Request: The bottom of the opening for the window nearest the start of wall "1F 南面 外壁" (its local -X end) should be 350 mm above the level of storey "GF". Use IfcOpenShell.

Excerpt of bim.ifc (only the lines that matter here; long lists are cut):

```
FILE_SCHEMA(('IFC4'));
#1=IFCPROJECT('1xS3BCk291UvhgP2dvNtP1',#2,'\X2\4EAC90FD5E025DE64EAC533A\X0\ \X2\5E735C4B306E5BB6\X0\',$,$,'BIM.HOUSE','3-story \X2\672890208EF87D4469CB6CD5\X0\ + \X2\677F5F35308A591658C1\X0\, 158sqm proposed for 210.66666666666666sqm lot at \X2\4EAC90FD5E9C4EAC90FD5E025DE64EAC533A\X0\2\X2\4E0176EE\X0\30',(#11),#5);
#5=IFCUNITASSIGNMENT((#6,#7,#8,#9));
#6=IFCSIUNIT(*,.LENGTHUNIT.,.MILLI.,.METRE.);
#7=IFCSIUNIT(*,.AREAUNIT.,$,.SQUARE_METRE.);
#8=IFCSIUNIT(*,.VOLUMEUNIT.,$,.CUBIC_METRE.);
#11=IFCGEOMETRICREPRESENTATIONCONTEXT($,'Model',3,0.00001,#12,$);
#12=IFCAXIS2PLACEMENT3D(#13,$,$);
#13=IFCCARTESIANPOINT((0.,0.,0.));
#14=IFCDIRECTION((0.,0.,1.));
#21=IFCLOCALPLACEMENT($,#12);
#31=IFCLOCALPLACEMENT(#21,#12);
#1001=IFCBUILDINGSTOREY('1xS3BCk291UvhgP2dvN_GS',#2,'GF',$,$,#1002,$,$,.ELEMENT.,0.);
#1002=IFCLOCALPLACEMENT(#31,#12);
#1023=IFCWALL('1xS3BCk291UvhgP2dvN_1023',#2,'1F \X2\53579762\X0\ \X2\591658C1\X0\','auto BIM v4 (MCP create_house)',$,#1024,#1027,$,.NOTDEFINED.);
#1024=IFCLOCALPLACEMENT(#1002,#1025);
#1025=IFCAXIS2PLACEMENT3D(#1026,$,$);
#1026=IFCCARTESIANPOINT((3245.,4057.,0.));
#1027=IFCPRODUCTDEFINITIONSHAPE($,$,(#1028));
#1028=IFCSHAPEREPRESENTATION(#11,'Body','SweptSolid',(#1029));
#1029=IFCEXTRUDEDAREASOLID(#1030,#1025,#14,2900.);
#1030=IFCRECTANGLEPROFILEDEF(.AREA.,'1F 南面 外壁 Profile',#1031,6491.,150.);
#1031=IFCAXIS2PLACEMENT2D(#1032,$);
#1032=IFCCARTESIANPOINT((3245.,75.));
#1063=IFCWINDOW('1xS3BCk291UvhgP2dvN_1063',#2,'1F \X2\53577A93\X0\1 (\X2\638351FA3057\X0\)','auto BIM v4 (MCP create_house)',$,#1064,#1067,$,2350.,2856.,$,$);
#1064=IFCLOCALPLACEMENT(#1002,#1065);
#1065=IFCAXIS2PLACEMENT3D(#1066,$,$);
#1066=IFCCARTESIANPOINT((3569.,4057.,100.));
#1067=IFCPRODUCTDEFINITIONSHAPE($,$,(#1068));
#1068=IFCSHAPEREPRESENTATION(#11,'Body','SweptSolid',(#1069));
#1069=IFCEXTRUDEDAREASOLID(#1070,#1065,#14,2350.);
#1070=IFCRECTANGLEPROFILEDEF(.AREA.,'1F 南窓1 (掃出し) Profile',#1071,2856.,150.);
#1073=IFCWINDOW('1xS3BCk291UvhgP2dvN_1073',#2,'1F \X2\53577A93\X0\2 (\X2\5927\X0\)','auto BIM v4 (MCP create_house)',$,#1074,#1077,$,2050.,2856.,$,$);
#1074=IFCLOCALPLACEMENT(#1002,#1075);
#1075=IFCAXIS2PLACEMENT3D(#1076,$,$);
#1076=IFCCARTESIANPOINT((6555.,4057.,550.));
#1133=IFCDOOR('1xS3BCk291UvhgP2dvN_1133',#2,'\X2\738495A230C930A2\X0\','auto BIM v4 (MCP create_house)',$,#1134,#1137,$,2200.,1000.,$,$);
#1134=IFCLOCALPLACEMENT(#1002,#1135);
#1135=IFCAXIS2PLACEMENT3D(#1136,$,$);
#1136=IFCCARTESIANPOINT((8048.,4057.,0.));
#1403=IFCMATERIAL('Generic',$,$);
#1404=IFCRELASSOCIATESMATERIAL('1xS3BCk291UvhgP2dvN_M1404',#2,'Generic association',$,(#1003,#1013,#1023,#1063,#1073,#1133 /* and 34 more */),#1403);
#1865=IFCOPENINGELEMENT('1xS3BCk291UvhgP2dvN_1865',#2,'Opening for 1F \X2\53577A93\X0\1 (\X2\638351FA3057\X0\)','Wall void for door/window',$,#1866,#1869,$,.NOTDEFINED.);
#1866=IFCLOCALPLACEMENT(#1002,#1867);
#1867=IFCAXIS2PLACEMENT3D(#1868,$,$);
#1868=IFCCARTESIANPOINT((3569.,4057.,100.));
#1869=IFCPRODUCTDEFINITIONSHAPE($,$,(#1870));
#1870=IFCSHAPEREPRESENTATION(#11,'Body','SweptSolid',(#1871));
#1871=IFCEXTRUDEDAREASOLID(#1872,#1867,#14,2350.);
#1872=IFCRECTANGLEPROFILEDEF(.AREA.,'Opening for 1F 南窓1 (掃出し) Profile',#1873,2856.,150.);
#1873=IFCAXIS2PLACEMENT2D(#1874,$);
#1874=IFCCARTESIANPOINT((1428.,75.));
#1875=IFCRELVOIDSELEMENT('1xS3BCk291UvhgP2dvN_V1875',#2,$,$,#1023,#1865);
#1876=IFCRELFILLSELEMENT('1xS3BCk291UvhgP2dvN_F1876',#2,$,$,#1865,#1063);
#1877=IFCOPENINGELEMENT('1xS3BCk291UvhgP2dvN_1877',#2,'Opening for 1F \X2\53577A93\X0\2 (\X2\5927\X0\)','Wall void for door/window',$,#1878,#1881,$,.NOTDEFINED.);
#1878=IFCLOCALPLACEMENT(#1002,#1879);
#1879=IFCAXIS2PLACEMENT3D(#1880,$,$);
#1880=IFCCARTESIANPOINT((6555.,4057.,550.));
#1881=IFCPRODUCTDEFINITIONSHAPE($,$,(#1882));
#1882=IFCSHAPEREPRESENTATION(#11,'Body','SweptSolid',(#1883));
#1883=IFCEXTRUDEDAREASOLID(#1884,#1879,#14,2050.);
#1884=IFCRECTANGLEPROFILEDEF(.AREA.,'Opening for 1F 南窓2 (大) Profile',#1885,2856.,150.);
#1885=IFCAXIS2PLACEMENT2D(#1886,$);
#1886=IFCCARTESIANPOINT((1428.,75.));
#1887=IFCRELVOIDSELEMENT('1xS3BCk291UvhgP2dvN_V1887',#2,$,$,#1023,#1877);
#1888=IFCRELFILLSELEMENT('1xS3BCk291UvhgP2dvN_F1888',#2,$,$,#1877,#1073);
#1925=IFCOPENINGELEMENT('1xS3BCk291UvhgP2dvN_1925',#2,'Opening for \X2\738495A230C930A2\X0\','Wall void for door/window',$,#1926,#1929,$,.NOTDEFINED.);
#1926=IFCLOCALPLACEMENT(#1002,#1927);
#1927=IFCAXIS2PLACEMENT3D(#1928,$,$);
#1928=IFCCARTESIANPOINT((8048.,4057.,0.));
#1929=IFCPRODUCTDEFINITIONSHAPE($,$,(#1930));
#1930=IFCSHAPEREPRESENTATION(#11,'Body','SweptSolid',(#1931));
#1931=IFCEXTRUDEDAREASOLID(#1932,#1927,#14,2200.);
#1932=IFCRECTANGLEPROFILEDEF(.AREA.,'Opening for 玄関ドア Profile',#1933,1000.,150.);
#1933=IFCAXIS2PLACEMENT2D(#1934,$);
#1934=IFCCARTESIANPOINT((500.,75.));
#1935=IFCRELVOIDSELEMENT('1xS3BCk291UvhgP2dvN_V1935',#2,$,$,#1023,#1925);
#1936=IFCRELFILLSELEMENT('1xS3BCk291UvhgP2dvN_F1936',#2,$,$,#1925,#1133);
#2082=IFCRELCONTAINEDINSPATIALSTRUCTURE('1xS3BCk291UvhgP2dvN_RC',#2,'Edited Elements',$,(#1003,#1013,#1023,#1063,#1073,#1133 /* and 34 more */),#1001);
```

```python
import numpy as np
import ifcopenshell
import ifcopenshell.api.geometry
import ifcopenshell.geom
import ifcopenshell.util.element
import ifcopenshell.util.placement
import ifcopenshell.util.shape
import ifcopenshell.util.unit

model = ifcopenshell.open("bim.ifc")
unit_scale = ifcopenshell.util.unit.calculate_unit_scale(model)

window = model.by_guid("1xS3BCk291UvhgP2dvN_1063")
opening = window.FillsVoids[0].RelatingOpeningElement
storey = ifcopenshell.util.element.get_container(window, ifc_class="IfcBuildingStorey")
level = ifcopenshell.util.placement.get_local_placement(storey.ObjectPlacement)[2, 3]

# The opening's origin need not be at the sill, so measure its lowest point.
shape = ifcopenshell.geom.create_shape(ifcopenshell.geom.settings(), opening)
bottom = ifcopenshell.util.shape.get_shape_bottom_elevation(shape, shape.geometry) / unit_scale
dz = level + 350.0 - bottom

shift = np.array([0.0, 0.0, dz])
# The window is not placed relative to its opening, so move both.
for product in (opening, window):
    matrix = ifcopenshell.util.placement.get_local_placement(product.ObjectPlacement)
    matrix[:3, 3] += shift
    ifcopenshell.api.geometry.edit_object_placement(model, product=product, matrix=matrix, is_si=False)

print(f"moved by {dz * unit_scale:+.3f} m")

model.write("bim_rev.ifc")
```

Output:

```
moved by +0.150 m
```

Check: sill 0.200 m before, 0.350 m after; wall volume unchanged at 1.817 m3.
